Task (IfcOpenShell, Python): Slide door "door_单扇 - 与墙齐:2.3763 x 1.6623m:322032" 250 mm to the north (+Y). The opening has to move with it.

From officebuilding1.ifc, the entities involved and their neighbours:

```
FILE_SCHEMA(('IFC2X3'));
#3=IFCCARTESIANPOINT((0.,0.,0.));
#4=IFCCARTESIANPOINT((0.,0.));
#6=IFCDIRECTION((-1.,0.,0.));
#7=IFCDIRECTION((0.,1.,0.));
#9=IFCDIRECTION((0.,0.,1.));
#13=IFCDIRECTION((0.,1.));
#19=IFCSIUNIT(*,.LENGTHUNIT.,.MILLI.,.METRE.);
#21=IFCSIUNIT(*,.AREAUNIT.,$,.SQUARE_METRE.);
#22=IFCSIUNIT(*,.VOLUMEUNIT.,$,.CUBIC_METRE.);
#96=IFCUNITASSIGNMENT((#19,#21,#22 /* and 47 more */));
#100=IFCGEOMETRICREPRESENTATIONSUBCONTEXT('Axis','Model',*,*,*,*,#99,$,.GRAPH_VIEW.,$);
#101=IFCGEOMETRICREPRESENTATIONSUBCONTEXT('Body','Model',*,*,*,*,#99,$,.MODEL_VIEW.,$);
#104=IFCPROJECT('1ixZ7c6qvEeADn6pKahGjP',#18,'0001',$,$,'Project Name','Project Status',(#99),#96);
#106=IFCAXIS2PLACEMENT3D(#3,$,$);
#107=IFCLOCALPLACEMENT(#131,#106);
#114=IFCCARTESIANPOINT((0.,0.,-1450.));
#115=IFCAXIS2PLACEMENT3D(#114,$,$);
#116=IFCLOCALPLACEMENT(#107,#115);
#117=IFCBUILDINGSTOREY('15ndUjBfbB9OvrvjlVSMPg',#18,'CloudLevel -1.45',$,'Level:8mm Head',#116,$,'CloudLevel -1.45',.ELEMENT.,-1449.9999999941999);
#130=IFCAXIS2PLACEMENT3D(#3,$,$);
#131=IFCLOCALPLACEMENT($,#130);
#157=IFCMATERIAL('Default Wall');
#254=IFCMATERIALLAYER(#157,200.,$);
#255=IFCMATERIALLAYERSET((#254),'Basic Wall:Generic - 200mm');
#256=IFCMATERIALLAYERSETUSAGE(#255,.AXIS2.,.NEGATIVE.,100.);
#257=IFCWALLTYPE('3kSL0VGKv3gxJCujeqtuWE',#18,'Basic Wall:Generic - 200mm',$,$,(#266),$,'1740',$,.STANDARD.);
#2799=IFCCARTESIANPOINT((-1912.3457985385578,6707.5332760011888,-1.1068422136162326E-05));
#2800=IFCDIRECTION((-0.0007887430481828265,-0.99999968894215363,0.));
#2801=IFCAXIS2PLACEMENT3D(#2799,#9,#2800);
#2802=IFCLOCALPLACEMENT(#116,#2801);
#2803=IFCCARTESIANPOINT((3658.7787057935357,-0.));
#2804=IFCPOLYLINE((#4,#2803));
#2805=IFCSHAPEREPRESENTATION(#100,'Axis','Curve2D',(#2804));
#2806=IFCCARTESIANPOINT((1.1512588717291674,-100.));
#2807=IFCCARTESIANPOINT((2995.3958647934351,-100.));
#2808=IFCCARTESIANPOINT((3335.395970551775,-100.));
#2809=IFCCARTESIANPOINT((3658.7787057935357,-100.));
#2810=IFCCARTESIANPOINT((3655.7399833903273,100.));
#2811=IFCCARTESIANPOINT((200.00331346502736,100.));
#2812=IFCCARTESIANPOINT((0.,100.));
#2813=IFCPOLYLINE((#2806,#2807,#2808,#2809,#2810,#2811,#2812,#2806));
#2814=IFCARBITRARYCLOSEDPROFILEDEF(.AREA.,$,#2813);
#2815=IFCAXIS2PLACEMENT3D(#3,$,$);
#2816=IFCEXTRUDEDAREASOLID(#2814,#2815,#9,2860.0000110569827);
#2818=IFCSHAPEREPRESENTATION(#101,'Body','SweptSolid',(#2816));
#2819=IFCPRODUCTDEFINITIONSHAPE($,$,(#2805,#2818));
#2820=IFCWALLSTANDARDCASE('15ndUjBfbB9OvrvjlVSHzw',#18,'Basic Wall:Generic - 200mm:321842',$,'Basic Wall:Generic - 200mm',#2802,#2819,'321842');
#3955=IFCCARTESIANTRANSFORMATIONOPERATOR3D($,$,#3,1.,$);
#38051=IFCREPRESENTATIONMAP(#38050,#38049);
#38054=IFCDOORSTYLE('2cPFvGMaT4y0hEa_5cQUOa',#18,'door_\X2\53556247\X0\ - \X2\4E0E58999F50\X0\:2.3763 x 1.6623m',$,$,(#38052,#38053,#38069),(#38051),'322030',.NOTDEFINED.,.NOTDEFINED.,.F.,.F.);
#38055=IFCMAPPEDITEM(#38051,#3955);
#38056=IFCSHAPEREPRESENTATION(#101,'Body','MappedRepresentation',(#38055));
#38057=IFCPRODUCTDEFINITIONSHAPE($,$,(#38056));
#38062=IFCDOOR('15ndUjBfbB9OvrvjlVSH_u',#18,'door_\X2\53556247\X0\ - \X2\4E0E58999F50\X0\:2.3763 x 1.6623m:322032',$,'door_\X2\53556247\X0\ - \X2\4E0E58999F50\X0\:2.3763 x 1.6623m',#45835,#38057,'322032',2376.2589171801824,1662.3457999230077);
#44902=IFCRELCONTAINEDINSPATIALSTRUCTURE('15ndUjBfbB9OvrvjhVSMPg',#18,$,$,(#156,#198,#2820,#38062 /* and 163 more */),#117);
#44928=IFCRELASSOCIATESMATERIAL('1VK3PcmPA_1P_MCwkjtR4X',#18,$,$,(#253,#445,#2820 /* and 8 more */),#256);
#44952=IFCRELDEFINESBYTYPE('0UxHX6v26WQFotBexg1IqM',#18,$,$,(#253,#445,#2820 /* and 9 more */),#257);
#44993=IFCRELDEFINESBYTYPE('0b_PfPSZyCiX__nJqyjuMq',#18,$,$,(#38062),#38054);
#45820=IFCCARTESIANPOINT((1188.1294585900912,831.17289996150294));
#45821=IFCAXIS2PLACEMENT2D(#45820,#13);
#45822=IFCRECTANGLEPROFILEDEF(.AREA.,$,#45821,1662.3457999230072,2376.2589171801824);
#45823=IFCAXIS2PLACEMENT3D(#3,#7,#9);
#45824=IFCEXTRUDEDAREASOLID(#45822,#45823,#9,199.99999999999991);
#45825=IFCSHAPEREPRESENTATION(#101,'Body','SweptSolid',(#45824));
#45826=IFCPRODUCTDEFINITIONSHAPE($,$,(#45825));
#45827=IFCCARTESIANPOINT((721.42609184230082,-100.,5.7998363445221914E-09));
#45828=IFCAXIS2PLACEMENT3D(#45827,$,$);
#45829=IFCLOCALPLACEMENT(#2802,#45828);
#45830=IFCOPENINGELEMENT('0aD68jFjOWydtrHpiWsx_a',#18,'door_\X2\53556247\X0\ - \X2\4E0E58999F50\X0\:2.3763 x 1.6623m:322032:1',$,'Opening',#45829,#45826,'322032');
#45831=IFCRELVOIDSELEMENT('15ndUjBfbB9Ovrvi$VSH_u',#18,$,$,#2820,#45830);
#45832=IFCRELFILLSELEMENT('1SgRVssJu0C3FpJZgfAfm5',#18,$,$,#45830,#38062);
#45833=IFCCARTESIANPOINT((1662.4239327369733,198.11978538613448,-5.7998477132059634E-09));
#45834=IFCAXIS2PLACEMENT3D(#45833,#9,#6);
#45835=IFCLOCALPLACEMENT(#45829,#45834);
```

```python
import ifcopenshell
import ifcopenshell.api.geometry
import ifcopenshell.util.placement

model = ifcopenshell.open("officebuilding1.ifc")

door = model.by_id(38062)
opening = door.FillsVoids[0].RelatingOpeningElement
wall = opening.VoidsElements[0].RelatingBuildingElement

wall_matrix = ifcopenshell.util.placement.get_local_placement(wall.ObjectPlacement)
shift = wall_matrix[:3, 0] * -250.0
before = ifcopenshell.util.placement.get_local_placement(door.ObjectPlacement)[:3, 3].copy()

# The door is placed relative to its opening, so it follows when the opening moves.
matrix = ifcopenshell.util.placement.get_local_placement(opening.ObjectPlacement)
matrix[:3, 3] += shift
ifcopenshell.api.geometry.edit_object_placement(
    model, product=opening, matrix=matrix, is_si=False, should_transform_children=True
)

after = ifcopenshell.util.placement.get_local_placement(door.ObjectPlacement)[:3, 3]
print("door moved by", (after - before).round(3) + 0.0)

model.write("officebuilding1-out.ifc")
```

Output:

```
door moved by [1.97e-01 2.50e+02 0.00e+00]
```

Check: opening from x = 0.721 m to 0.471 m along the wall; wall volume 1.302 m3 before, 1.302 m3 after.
